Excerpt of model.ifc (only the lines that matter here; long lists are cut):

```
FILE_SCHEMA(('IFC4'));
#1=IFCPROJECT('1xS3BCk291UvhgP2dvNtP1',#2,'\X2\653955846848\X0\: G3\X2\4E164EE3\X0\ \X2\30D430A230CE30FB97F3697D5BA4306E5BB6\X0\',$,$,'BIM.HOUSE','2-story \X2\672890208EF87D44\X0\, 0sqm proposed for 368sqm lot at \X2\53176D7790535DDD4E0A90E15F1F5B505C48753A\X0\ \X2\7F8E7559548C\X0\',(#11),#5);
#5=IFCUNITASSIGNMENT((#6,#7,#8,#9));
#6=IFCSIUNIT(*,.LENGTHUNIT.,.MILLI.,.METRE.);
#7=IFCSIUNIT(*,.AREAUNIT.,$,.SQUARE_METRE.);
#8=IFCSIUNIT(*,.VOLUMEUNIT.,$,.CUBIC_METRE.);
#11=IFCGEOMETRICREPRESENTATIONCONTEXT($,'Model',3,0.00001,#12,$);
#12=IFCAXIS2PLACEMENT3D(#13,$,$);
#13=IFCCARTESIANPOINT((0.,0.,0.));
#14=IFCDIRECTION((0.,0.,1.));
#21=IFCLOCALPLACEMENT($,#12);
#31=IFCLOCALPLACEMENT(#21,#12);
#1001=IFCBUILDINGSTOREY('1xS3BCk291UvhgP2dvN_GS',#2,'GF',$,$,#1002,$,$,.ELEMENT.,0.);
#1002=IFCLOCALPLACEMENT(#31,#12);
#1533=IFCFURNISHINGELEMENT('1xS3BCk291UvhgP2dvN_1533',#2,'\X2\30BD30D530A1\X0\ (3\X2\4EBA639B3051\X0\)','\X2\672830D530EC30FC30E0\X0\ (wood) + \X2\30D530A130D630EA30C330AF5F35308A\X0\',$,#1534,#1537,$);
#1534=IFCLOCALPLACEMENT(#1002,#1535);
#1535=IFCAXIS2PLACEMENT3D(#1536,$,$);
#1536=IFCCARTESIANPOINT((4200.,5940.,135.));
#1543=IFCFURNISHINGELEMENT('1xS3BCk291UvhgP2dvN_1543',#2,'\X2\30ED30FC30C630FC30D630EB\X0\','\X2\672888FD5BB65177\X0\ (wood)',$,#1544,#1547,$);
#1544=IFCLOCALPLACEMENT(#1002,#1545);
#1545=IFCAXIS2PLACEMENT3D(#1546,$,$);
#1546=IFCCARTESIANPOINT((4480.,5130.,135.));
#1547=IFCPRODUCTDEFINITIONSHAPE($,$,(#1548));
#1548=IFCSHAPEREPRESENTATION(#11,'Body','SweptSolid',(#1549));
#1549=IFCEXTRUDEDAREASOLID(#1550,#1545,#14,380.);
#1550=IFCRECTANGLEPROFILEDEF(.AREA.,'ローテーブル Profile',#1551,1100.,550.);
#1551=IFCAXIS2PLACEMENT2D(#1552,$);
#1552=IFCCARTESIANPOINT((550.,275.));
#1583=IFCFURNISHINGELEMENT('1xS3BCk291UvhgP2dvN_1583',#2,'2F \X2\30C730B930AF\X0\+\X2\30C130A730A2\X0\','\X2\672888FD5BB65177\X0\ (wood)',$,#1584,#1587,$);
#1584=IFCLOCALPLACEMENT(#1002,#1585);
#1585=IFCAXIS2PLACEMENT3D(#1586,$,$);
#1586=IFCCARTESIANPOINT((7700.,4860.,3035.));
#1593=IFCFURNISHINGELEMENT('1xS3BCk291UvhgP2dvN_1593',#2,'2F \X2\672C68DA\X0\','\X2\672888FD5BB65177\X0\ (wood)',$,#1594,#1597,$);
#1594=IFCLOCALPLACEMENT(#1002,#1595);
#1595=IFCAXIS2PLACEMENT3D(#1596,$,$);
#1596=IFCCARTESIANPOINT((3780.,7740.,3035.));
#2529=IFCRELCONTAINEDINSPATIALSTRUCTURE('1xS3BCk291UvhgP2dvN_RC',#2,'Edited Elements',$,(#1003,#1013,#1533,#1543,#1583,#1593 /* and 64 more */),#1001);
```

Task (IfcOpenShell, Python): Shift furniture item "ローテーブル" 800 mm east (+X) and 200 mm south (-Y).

```python
import ifcopenshell
import ifcopenshell.api.geometry
import ifcopenshell.util.placement

model = ifcopenshell.open("model.ifc")

item = model.by_id(1543)
matrix = ifcopenshell.util.placement.get_local_placement(item.ObjectPlacement)
matrix[0, 3] += 800.0
matrix[1, 3] -= 200.0
ifcopenshell.api.geometry.edit_object_placement(model, product=item, matrix=matrix, is_si=False)

print(ifcopenshell.util.placement.get_local_placement(item.ObjectPlacement).round(3) + 0.0)

model.write("model-out.ifc")
```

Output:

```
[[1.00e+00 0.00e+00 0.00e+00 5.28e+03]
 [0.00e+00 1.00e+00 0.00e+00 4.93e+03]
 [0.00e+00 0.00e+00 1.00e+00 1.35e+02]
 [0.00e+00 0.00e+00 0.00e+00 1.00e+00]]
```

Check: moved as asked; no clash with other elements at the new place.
